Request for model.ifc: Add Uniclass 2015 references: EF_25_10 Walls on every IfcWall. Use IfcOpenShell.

First a look at what the model holds.

```python
import ifcopenshell

model = ifcopenshell.open("model.ifc")
print(model.schema)
print("classifications:", [c.Name for c in model.by_type("IfcClassification")])
for ifc_class in ("IfcDoor", "IfcRoof", "IfcStair", "IfcWall", "IfcWindow"):
    print(ifc_class, len(model.by_type(ifc_class)))
```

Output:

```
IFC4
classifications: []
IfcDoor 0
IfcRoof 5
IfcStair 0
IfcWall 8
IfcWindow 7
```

```python
import ifcopenshell
import ifcopenshell.api.classification

model = ifcopenshell.open("model.ifc")

system = ifcopenshell.api.classification.add_classification(model, classification="Uniclass 2015")

codes = {
    "IfcWall": ("EF_25_10", "Walls"),
}
for ifc_class, (code, name) in codes.items():
    products = model.by_type(ifc_class)
    ifcopenshell.api.classification.add_reference(
        model, products=products, classification=system, identification=code, name=name
    )
    print(code, len(products))

model.write("model-out.ifc")
```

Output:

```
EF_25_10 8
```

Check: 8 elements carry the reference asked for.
